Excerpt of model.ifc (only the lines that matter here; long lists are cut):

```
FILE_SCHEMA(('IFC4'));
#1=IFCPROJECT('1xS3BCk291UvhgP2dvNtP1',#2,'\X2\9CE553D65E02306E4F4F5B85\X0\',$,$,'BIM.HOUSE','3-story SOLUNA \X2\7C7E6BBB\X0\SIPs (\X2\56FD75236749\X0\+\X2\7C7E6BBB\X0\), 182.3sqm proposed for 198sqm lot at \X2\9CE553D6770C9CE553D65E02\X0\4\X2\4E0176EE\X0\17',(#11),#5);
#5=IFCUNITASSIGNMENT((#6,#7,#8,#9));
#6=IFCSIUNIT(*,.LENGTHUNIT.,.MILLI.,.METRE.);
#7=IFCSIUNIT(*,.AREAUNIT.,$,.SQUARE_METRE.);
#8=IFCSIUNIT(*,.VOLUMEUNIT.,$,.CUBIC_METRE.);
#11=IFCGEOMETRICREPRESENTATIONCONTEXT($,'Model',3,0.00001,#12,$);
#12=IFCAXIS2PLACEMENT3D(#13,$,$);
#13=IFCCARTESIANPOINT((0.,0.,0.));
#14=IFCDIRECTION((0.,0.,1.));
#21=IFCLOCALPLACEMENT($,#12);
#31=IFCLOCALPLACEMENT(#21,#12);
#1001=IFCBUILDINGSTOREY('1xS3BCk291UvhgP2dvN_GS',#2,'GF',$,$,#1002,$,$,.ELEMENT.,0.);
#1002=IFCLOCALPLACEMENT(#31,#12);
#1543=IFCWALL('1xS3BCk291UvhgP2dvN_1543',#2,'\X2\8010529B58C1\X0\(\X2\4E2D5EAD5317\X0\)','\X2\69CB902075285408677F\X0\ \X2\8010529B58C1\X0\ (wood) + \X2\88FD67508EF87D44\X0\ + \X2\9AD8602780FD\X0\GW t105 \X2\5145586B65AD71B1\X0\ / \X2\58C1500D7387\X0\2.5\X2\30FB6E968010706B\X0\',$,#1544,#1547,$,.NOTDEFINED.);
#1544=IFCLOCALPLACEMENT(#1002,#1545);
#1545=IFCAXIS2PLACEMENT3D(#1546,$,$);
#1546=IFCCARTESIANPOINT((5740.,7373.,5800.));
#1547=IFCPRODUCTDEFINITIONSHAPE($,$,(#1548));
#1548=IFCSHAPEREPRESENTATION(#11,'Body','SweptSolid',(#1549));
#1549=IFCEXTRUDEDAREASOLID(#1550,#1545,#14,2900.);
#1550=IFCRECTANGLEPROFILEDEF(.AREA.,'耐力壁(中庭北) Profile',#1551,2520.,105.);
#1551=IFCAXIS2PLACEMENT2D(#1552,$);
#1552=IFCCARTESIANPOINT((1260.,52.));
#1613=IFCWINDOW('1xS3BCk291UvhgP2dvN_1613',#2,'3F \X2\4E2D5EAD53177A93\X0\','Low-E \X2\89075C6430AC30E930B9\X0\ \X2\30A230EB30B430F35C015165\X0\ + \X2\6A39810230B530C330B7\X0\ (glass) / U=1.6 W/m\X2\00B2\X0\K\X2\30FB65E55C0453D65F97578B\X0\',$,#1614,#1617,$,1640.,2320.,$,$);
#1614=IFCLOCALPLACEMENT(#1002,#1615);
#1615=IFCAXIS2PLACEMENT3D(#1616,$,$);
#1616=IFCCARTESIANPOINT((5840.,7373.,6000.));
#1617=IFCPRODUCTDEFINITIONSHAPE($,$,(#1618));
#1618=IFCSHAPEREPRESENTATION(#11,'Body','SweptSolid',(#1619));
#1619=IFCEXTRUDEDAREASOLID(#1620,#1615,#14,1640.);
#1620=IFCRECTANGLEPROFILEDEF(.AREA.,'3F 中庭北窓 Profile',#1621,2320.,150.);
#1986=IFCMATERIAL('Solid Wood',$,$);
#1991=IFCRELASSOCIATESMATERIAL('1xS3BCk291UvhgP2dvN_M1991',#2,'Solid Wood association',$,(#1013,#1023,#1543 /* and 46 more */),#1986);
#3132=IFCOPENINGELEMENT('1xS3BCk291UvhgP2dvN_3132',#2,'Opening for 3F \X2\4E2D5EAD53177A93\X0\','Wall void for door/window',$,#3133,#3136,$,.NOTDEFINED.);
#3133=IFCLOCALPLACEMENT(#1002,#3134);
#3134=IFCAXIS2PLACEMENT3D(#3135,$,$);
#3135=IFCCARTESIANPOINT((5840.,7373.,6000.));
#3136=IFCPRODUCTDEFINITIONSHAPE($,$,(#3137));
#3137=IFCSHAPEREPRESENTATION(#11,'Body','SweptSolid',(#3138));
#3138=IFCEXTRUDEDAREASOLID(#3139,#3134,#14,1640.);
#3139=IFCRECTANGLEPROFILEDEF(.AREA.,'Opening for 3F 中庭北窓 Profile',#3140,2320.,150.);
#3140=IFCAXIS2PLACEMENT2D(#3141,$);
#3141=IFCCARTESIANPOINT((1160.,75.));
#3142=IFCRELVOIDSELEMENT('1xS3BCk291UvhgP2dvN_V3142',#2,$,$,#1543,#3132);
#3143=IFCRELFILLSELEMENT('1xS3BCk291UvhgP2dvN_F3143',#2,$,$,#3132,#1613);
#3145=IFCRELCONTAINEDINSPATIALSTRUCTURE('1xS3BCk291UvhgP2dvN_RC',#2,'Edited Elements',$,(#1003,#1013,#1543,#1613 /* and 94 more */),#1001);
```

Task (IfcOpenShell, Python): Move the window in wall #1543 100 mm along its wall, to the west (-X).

```python
import ifcopenshell
import ifcopenshell.api.geometry
import ifcopenshell.util.placement

model = ifcopenshell.open("model.ifc")

window = model.by_id(1613)
opening = window.FillsVoids[0].RelatingOpeningElement
wall = opening.VoidsElements[0].RelatingBuildingElement

wall_matrix = ifcopenshell.util.placement.get_local_placement(wall.ObjectPlacement)
shift = wall_matrix[:3, 0] * -100.0
before = ifcopenshell.util.placement.get_local_placement(window.ObjectPlacement)[:3, 3].copy()

# The window is not placed relative to its opening, so move both.
for product in (opening, window):
    matrix = ifcopenshell.util.placement.get_local_placement(product.ObjectPlacement)
    matrix[:3, 3] += shift
    ifcopenshell.api.geometry.edit_object_placement(model, product=product, matrix=matrix, is_si=False)

after = ifcopenshell.util.placement.get_local_placement(window.ObjectPlacement)[:3, 3]
print("window moved by", (after - before).round(3) + 0.0)

model.write("model_edited.ifc")
```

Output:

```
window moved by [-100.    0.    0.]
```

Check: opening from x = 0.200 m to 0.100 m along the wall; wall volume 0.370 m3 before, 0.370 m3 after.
